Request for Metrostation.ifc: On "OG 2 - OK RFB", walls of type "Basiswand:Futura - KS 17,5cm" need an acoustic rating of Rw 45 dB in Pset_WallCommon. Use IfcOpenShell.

First a look at what the model holds.

```python
import ifcopenshell
import ifcopenshell.util.element

model = ifcopenshell.open("Metrostation.ifc")
print(model.schema)
storey = next(s for s in model.by_type("IfcBuildingStorey") if s.Name == "OG 2 - OK RFB")
walls = [e for e in ifcopenshell.util.element.get_decomposition(storey) if e.is_a("IfcWall")]
seen = {}
for e in walls:
    element_type = ifcopenshell.util.element.get_type(e)
    key = (element_type.Name if element_type != e and element_type else None, ifcopenshell.util.element.get_pset(e, "Pset_WallCommon", "AcousticRating"))
    seen[key] = seen.get(key, 0) + 1
for (name, value), count in sorted(seen.items(), key=str):
    print(count, "x", name, "|", value)
```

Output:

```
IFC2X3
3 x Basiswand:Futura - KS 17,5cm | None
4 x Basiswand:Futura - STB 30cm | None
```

```python
import ifcopenshell
import ifcopenshell.api.pset
import ifcopenshell.util.element

model = ifcopenshell.open("Metrostation.ifc")

storey = next(s for s in model.by_type("IfcBuildingStorey") if s.Name == "OG 2 - OK RFB")
walls = [e for e in ifcopenshell.util.element.get_decomposition(storey) if e.is_a("IfcWall")]

count = 0
for e in walls:
    element_type = ifcopenshell.util.element.get_type(e)
    if element_type in (None, e) or element_type.Name != "Basiswand:Futura - KS 17,5cm":
        continue
    # add_pset returns the element's existing set when there is one.
    pset = ifcopenshell.api.pset.add_pset(model, product=e, name="Pset_WallCommon")
    ifcopenshell.api.pset.edit_pset(model, pset=pset, properties={"AcousticRating": "Rw 45 dB"})
    count += 1

print(count, "walls updated")

model.write("Metrostation_edited.ifc")
```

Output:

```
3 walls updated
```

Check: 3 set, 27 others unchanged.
